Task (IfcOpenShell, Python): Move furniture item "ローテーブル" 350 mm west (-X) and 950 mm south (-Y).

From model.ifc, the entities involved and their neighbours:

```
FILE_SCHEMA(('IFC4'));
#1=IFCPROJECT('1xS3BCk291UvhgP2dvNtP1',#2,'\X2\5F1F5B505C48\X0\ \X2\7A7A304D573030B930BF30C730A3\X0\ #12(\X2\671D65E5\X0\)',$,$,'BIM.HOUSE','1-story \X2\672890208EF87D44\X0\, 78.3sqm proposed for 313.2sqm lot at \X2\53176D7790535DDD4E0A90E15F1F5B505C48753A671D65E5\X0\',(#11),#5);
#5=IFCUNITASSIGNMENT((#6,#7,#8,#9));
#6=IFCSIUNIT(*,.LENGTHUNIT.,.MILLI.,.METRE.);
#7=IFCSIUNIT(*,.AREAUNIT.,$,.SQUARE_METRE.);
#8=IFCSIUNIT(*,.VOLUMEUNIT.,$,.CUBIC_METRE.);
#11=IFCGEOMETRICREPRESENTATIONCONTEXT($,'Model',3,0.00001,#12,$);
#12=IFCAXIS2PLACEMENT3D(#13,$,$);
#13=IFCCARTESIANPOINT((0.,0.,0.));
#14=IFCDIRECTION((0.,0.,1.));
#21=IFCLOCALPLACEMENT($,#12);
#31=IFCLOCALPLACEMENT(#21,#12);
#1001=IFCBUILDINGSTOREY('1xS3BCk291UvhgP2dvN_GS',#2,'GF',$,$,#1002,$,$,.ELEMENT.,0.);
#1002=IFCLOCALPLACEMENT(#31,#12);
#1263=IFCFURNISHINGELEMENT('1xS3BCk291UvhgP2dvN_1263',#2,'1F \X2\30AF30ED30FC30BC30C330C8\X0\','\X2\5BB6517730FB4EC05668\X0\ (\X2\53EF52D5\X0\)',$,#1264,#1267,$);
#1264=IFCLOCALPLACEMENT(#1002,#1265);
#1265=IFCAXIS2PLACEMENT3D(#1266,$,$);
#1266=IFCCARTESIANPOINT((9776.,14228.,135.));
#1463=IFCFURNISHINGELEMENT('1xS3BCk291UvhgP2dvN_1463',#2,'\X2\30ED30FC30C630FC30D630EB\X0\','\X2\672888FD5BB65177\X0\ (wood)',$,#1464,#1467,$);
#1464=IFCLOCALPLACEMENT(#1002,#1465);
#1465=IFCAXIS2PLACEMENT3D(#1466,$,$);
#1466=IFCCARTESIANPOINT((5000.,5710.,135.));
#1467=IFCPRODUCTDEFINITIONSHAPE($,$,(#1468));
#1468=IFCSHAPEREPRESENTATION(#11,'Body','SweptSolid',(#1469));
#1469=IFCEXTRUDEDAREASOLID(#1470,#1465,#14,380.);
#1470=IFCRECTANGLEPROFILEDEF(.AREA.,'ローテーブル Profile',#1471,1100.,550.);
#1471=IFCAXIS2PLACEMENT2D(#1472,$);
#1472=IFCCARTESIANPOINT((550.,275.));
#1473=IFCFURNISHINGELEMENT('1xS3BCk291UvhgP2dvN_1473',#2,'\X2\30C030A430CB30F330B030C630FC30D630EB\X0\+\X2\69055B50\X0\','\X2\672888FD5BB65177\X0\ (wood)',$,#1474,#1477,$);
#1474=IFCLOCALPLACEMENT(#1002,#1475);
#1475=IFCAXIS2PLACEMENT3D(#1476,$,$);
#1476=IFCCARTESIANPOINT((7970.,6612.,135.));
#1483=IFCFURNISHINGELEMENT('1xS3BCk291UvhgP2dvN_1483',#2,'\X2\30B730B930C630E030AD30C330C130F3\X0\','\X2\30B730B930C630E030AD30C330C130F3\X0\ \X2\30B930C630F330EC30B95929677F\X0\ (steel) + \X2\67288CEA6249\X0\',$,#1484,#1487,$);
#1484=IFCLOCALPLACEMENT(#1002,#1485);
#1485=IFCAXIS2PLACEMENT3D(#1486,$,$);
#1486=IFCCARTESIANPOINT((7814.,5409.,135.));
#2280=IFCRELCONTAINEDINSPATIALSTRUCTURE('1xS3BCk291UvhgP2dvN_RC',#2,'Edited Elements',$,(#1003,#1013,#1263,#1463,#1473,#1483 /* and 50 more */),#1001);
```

```python
import ifcopenshell
import ifcopenshell.api.geometry
import ifcopenshell.util.placement
import ifcopenshell.util.unit

model = ifcopenshell.open("model.ifc")
unit_scale = ifcopenshell.util.unit.calculate_unit_scale(model)

item = model.by_id(1463)
matrix = ifcopenshell.util.placement.get_local_placement(item.ObjectPlacement)
matrix[0, 3] -= 0.35 / unit_scale
matrix[1, 3] -= 0.95 / unit_scale
ifcopenshell.api.geometry.edit_object_placement(model, product=item, matrix=matrix, is_si=False)

print(ifcopenshell.util.placement.get_local_placement(item.ObjectPlacement).round(3) + 0.0)

model.write("model_updated.ifc")
```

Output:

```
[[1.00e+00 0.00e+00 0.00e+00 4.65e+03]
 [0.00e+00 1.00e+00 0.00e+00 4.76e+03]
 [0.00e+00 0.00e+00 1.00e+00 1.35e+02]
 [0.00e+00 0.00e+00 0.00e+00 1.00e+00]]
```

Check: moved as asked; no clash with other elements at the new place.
